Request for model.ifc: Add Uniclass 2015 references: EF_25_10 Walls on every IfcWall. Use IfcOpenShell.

First a look at what the model holds.

```python
import ifcopenshell

model = ifcopenshell.open("model.ifc")
print(model.schema)
print("classifications:", [c.Name for c in model.by_type("IfcClassification")])
for ifc_class in ("IfcDoor", "IfcRoof", "IfcStair", "IfcWall", "IfcWindow"):
    print(ifc_class, len(model.by_type(ifc_class)))
```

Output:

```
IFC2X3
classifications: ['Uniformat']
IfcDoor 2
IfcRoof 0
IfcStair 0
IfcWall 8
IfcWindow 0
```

```python
import ifcopenshell
import ifcopenshell.api.classification

model = ifcopenshell.open("model.ifc")

# IFC2X3 requires Source and Edition and has no link from the project to the system.
system = model.create_entity("IfcClassification", Source="NBS", Edition="2015", Name="Uniclass 2015")

codes = {
    "IfcWall": ("EF_25_10", "Walls"),
}
for ifc_class, (code, name) in codes.items():
    products = model.by_type(ifc_class)
    ifcopenshell.api.classification.add_reference(
        model, products=products, classification=system, identification=code, name=name
    )
    print(code, len(products))

model.write("model_v2.ifc")
```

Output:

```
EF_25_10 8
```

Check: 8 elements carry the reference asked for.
